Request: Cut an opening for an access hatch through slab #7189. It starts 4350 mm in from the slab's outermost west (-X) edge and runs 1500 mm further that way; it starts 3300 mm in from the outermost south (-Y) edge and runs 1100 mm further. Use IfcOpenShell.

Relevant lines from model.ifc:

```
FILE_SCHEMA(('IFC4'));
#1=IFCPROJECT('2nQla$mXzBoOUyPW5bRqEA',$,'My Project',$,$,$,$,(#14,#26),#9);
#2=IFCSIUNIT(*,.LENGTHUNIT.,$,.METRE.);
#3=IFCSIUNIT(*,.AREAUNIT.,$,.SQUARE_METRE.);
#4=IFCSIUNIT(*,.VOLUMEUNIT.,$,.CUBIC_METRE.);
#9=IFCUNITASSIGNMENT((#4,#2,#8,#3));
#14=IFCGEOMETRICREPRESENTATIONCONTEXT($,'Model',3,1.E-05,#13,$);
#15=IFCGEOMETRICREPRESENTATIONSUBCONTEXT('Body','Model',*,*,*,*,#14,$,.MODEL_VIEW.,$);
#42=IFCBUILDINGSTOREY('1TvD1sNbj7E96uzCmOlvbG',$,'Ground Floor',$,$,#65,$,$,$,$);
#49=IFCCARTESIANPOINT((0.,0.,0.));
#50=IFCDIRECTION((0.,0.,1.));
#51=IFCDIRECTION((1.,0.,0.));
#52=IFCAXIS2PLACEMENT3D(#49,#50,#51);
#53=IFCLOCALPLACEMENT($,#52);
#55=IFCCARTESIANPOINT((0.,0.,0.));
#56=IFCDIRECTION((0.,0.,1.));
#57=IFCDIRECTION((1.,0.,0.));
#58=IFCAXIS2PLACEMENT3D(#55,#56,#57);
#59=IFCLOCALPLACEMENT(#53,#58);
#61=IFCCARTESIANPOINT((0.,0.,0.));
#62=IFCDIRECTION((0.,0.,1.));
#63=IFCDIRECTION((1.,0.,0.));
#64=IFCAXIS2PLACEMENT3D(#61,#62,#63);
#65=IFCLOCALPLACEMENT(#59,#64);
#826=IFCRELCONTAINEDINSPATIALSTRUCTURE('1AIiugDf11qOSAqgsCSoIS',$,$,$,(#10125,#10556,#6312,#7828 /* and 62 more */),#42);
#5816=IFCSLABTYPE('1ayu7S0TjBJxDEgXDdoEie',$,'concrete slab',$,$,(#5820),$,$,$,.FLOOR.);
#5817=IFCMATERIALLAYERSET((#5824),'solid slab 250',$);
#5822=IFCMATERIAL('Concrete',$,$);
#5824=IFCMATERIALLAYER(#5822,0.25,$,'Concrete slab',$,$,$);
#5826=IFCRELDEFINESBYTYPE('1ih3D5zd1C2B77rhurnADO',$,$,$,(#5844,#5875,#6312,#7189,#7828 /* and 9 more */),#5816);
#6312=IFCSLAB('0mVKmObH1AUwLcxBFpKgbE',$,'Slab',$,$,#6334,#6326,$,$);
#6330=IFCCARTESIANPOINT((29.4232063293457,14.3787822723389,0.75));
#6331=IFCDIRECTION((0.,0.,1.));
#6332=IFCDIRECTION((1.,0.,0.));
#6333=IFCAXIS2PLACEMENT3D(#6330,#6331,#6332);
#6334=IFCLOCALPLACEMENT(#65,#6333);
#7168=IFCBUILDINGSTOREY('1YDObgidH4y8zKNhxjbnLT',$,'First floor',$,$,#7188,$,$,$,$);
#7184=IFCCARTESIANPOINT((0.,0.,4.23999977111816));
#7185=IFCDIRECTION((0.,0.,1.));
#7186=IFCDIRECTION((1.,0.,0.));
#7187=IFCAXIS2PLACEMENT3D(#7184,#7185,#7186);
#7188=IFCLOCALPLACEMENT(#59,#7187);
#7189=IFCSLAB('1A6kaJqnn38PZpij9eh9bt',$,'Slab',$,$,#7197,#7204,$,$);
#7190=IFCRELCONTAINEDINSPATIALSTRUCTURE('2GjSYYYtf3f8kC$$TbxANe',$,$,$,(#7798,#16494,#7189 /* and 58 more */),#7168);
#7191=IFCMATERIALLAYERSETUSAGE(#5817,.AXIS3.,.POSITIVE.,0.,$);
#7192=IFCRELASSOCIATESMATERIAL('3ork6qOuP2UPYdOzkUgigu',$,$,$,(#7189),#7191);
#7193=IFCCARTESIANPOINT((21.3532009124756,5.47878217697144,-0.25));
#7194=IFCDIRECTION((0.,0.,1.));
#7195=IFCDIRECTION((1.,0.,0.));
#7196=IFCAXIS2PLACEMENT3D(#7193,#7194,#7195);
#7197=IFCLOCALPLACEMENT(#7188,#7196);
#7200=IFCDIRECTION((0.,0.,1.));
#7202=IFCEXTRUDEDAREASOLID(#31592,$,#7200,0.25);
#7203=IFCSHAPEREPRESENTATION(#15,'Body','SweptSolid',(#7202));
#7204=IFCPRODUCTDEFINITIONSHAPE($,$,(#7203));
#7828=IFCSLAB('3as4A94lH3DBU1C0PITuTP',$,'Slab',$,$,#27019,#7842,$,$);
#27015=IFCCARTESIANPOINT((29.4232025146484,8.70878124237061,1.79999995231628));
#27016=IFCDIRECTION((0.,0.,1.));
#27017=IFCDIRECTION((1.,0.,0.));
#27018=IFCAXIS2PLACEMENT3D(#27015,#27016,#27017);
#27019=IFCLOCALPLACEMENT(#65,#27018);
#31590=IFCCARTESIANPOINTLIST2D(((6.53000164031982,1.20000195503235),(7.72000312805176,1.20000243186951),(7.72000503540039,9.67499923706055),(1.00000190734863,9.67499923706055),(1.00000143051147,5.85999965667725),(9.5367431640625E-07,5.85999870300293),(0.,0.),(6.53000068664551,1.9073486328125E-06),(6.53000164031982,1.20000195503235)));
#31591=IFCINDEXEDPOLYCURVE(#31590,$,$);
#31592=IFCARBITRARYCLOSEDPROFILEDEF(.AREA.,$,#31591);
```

```python
import numpy as np
import ifcopenshell
import ifcopenshell.api.feature
import ifcopenshell.api.geometry
import ifcopenshell.api.root
import ifcopenshell.geom
import ifcopenshell.util.placement
import ifcopenshell.util.representation
import ifcopenshell.util.shape
import ifcopenshell.util.unit

model = ifcopenshell.open("model.ifc")
unit_scale = ifcopenshell.util.unit.calculate_unit_scale(model)
settings = ifcopenshell.geom.settings()


def volume(element):
    """Net volume in cubic metres, openings subtracted."""
    shape = ifcopenshell.geom.create_shape(settings, element)
    return ifcopenshell.util.shape.get_volume(shape.geometry)


slab = model.by_guid("1A6kaJqnn38PZpij9eh9bt")
before = volume(slab)

# Extent in the slab's own axes, in metres. The edges named are its -X and -Y sides.
slab_shape = ifcopenshell.geom.create_shape(settings, slab)
vertices = ifcopenshell.util.shape.get_vertices(slab_shape.geometry)
x_min, y_min, bottom = vertices.min(axis=0)
top = vertices[:, 2].max()

opening = ifcopenshell.api.root.create_entity(model, ifc_class="IfcOpeningElement", name="Access hatch opening", predefined_type="OPENING")
context = ifcopenshell.util.representation.get_context(model, "Model", "Body", "MODEL_VIEW")
width, depth = 1.5, 1.1
outline = [(0.0, 0.0), (width, 0.0), (width, depth), (0.0, depth), (0.0, 0.0)]
# Overshoot both faces by 50 mm so the cut is clean.
shape = ifcopenshell.api.geometry.add_slab_representation(
    model, context=context, depth=top - bottom + 0.1, polyline=outline
)
ifcopenshell.api.geometry.assign_representation(model, product=opening, representation=shape)

matrix = ifcopenshell.util.placement.get_local_placement(slab.ObjectPlacement)
matrix[:, 3] = matrix @ np.append(np.array([x_min + 4.35, y_min + 3.3, bottom - 0.05]) / unit_scale, 1.0)
ifcopenshell.api.geometry.edit_object_placement(model, product=opening, matrix=matrix, is_si=False)
ifcopenshell.api.feature.add_feature(model, feature=opening, element=slab)

after = volume(slab)

print(f"slab volume {before:.3f} -> {after:.3f} m3")

model.write("model_rev.ifc")
```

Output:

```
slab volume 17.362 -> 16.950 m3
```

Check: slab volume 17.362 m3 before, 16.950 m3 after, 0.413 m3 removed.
